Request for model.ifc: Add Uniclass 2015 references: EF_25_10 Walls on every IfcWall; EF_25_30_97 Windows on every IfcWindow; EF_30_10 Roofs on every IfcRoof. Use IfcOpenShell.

First a look at what the model holds.

```python
import ifcopenshell

model = ifcopenshell.open("model.ifc")
print(model.schema)
print("classifications:", [c.Name for c in model.by_type("IfcClassification")])
for ifc_class in ("IfcDoor", "IfcRoof", "IfcStair", "IfcWall", "IfcWindow"):
    print(ifc_class, len(model.by_type(ifc_class)))
```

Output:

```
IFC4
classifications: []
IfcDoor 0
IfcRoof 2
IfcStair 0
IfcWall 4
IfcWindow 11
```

```python
import ifcopenshell
import ifcopenshell.api.classification

model = ifcopenshell.open("model.ifc")

system = ifcopenshell.api.classification.add_classification(model, classification="Uniclass 2015")

codes = {
    "IfcWall": ("EF_25_10", "Walls"),
    "IfcWindow": ("EF_25_30_97", "Windows"),
    "IfcRoof": ("EF_30_10", "Roofs"),
}
for ifc_class, (code, name) in codes.items():
    products = model.by_type(ifc_class)
    ifcopenshell.api.classification.add_reference(
        model, products=products, classification=system, identification=code, name=name
    )
    print(code, len(products))

model.write("model_edited.ifc")
```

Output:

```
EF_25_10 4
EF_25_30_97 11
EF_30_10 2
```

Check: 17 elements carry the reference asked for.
